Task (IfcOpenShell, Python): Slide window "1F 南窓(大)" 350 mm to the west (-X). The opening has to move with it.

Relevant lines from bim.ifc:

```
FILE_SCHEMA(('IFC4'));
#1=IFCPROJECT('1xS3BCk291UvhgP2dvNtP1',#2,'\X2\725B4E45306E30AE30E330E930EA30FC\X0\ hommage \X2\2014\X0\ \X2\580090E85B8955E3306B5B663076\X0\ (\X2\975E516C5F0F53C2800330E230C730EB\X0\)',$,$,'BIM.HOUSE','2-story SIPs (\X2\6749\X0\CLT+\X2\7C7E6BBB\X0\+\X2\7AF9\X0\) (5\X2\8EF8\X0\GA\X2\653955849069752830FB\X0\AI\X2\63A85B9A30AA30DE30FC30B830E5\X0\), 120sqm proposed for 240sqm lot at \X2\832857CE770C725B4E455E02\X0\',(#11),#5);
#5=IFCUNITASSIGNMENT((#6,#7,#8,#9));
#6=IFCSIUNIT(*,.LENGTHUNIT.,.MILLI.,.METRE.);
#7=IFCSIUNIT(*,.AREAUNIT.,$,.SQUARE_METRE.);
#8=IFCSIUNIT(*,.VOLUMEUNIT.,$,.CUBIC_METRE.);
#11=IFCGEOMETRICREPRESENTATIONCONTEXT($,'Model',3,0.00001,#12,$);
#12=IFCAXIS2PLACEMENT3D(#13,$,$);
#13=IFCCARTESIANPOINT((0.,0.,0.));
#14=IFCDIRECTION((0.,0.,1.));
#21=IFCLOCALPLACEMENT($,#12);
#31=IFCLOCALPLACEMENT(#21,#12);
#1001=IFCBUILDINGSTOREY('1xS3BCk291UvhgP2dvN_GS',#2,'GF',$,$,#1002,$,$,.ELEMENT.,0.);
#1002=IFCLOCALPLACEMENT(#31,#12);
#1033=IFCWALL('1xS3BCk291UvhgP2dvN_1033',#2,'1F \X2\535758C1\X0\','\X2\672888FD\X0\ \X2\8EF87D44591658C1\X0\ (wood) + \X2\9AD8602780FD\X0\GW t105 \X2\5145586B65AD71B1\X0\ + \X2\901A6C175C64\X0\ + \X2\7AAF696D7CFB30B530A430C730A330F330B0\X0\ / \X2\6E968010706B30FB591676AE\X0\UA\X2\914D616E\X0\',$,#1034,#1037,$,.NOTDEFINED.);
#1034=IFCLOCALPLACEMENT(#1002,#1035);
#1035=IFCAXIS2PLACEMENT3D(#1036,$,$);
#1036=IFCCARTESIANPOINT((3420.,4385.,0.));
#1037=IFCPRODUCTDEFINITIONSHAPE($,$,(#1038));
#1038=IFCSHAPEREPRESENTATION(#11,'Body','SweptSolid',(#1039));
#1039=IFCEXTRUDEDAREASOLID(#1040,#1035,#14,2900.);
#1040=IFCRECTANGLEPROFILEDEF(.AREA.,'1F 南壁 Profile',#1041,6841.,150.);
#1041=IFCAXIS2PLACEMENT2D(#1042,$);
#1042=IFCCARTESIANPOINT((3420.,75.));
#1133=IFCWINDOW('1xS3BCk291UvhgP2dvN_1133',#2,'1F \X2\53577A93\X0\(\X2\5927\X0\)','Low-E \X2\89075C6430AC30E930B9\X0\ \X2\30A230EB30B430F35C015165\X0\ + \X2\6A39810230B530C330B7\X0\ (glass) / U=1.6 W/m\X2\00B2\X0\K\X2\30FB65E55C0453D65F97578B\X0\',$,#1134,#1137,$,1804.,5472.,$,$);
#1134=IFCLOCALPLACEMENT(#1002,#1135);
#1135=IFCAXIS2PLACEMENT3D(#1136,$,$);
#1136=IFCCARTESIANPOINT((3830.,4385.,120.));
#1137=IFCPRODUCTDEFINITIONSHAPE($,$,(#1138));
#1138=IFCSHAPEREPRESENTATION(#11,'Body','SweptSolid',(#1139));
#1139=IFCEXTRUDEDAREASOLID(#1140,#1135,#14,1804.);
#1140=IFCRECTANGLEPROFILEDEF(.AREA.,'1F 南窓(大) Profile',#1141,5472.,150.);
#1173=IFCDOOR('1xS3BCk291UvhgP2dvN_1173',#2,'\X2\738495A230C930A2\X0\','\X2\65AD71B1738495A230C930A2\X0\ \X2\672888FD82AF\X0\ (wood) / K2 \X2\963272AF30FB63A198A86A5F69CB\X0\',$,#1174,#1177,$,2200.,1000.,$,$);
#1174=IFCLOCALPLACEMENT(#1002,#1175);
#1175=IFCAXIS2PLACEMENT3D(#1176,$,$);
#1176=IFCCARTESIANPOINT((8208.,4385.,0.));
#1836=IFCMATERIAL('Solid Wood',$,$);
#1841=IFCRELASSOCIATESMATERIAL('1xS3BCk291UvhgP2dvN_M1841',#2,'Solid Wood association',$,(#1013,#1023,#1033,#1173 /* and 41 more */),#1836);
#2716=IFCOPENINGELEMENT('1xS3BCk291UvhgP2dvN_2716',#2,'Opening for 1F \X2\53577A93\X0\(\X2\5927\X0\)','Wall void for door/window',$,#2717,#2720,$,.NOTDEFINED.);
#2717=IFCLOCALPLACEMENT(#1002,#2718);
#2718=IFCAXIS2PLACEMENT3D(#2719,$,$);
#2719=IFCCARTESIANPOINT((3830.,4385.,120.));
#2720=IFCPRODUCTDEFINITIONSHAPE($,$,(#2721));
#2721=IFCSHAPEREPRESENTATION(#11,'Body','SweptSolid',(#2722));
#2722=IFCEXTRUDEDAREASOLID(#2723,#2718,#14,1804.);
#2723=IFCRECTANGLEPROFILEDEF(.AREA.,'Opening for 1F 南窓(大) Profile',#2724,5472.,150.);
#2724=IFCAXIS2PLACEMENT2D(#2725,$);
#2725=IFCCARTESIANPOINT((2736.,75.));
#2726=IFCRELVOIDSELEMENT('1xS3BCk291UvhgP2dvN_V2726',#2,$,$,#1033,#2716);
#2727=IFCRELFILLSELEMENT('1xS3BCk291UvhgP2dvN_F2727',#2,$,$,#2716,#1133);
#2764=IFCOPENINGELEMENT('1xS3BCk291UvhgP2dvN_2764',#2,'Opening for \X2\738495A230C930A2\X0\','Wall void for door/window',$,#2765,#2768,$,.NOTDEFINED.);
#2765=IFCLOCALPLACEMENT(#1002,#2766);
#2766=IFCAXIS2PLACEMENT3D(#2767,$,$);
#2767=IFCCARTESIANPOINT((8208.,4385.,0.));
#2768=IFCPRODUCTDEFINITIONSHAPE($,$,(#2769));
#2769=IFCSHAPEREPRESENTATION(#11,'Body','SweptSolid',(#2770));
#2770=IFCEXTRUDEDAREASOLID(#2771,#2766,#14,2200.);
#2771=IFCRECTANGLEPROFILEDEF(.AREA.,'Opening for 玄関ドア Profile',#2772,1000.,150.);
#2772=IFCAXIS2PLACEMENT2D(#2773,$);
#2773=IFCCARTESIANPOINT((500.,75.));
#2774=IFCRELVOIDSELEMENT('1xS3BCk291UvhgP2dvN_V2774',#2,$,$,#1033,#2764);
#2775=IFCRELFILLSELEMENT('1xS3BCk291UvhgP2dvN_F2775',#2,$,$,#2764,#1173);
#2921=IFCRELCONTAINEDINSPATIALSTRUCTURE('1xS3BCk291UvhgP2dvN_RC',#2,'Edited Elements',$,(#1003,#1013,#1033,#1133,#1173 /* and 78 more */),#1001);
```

```python
import ifcopenshell
import ifcopenshell.api.geometry
import ifcopenshell.util.placement
import ifcopenshell.util.unit

model = ifcopenshell.open("bim.ifc")
unit_scale = ifcopenshell.util.unit.calculate_unit_scale(model)

window = model.by_guid("1xS3BCk291UvhgP2dvN_1133")
opening = window.FillsVoids[0].RelatingOpeningElement
wall = opening.VoidsElements[0].RelatingBuildingElement

wall_matrix = ifcopenshell.util.placement.get_local_placement(wall.ObjectPlacement)
shift = wall_matrix[:3, 0] * -0.35 / unit_scale
before = ifcopenshell.util.placement.get_local_placement(window.ObjectPlacement)[:3, 3].copy()

# The window is not placed relative to its opening, so move both.
for product in (opening, window):
    matrix = ifcopenshell.util.placement.get_local_placement(product.ObjectPlacement)
    matrix[:3, 3] += shift
    ifcopenshell.api.geometry.edit_object_placement(model, product=product, matrix=matrix, is_si=False)

after = ifcopenshell.util.placement.get_local_placement(window.ObjectPlacement)[:3, 3]
print("window moved by", (after - before).round(3) + 0.0)

model.write("bim-out.ifc")
```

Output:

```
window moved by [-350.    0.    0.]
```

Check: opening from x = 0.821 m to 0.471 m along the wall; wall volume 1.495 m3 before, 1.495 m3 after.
